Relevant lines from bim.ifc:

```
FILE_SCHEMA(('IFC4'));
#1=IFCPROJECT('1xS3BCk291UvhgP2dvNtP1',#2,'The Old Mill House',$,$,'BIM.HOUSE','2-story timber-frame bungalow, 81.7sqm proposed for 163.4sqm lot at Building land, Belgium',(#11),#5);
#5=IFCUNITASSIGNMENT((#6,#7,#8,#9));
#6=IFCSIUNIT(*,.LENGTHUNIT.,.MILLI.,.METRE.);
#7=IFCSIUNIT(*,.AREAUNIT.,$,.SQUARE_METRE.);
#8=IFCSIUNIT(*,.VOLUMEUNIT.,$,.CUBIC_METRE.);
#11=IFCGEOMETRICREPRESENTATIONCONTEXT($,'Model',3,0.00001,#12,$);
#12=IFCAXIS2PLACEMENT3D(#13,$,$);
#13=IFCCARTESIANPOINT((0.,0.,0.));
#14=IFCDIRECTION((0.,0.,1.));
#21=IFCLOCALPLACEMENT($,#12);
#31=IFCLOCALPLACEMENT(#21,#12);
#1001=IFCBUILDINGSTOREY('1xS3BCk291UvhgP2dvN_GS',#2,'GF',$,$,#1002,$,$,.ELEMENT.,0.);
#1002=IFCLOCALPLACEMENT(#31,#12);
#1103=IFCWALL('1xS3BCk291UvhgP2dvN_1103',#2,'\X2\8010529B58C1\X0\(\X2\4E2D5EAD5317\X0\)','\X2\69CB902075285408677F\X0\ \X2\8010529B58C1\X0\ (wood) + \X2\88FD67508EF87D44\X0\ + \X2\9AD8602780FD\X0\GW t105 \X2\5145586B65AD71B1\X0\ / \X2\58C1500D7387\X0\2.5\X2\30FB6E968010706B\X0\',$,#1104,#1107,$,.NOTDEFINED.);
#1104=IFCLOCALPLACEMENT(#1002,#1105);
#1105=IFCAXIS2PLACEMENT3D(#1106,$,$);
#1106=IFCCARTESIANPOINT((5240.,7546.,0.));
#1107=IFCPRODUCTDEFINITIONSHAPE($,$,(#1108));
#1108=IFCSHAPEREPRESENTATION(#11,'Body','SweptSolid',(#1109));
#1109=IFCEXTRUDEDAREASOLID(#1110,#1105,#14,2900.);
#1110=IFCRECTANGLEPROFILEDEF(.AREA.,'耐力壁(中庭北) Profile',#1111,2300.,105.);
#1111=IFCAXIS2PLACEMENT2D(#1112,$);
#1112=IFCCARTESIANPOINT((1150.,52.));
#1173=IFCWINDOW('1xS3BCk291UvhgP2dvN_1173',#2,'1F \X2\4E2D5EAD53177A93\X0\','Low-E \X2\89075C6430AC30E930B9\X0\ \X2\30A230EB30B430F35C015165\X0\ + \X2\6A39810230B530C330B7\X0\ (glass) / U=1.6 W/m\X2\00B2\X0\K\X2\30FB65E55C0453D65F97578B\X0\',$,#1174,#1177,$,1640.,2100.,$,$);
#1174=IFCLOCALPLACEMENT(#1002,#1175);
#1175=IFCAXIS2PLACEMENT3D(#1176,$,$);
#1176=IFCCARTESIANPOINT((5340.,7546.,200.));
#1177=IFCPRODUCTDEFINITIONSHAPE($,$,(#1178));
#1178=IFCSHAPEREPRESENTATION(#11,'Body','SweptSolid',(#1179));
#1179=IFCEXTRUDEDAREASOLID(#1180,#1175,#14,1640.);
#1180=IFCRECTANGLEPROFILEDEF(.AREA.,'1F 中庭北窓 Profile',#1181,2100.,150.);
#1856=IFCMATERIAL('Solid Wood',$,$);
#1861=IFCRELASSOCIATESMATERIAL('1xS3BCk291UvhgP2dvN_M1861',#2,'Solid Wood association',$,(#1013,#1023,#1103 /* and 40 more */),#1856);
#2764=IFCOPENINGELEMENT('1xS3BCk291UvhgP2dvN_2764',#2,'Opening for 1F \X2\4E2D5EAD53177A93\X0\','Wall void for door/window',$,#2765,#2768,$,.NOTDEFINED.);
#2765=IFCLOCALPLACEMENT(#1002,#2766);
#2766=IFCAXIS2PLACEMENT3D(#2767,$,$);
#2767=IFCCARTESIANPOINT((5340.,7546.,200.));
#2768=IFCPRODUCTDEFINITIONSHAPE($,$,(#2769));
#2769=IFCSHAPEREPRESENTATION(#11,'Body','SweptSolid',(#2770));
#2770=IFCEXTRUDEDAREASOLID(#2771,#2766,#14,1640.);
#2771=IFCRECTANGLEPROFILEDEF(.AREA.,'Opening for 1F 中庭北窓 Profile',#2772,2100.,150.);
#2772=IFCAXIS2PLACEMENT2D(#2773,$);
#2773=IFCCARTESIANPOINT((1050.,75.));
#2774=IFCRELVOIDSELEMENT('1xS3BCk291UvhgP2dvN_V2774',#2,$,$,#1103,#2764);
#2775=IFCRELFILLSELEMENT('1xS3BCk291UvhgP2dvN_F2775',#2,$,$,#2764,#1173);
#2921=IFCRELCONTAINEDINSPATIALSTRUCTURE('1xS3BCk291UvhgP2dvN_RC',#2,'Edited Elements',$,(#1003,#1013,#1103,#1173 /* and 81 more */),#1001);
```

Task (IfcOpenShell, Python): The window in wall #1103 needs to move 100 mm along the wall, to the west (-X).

```python
import ifcopenshell
import ifcopenshell.api.geometry
import ifcopenshell.util.placement

model = ifcopenshell.open("bim.ifc")

window = model.by_guid("1xS3BCk291UvhgP2dvN_1173")
opening = window.FillsVoids[0].RelatingOpeningElement
wall = opening.VoidsElements[0].RelatingBuildingElement

wall_matrix = ifcopenshell.util.placement.get_local_placement(wall.ObjectPlacement)
shift = wall_matrix[:3, 0] * -100.0
before = ifcopenshell.util.placement.get_local_placement(window.ObjectPlacement)[:3, 3].copy()

# The window is not placed relative to its opening, so move both.
for product in (opening, window):
    matrix = ifcopenshell.util.placement.get_local_placement(product.ObjectPlacement)
    matrix[:3, 3] += shift
    ifcopenshell.api.geometry.edit_object_placement(model, product=product, matrix=matrix, is_si=False)

after = ifcopenshell.util.placement.get_local_placement(window.ObjectPlacement)[:3, 3]
print("window moved by", (after - before).round(3) + 0.0)

model.write("bim_v2.ifc")
```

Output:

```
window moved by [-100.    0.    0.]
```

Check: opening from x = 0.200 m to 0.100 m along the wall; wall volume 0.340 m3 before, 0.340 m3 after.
